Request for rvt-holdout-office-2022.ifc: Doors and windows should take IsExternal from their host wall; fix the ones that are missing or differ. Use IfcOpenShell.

First a look at what the model holds.

```python
import ifcopenshell
import ifcopenshell.util.element

model = ifcopenshell.open("rvt-holdout-office-2022.ifc")
print(model.schema)
seen = {}
for e in model.by_type("IfcDoor") + model.by_type("IfcWindow"):
    if not e.FillsVoids:
        continue
    host = e.FillsVoids[0].RelatingOpeningElement.VoidsElements[0].RelatingBuildingElement
    own = ifcopenshell.util.element.get_pset(e, f"Pset_{e.is_a()[3:].removesuffix('StandardCase')}Common", "IsExternal")
    wall = ifcopenshell.util.element.get_pset(host, "Pset_WallCommon", "IsExternal")
    seen[e.is_a(), own, wall] = seen.get((e.is_a(), own, wall), 0) + 1
for (cls, own, wall), count in sorted(seen.items(), key=str):
    print(count, cls, "IsExternal:", own, "| host wall:", wall)
```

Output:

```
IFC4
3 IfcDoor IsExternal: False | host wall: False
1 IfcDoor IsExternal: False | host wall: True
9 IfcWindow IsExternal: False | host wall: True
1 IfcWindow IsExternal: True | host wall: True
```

```python
import ifcopenshell
import ifcopenshell.api.pset
import ifcopenshell.util.element

model = ifcopenshell.open("rvt-holdout-office-2022.ifc")

count = 0
for ifc_class, pset_name in (("IfcDoor", "Pset_DoorCommon"), ("IfcWindow", "Pset_WindowCommon")):
    for e in model.by_type(ifc_class):
        if not e.FillsVoids:
            continue
        host = e.FillsVoids[0].RelatingOpeningElement.VoidsElements[0].RelatingBuildingElement
        external = ifcopenshell.util.element.get_pset(host, "Pset_WallCommon", "IsExternal")
        if external is None or ifcopenshell.util.element.get_pset(e, pset_name, "IsExternal") == external:
            continue
        pset = ifcopenshell.api.pset.add_pset(model, product=e, name=pset_name)
        ifcopenshell.api.pset.edit_pset(model, pset=pset, properties={"IsExternal": external})
        count += 1

print(count, "updated")

model.write("rvt-holdout-office-2022_updated.ifc")
```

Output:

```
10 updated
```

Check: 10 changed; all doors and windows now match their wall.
